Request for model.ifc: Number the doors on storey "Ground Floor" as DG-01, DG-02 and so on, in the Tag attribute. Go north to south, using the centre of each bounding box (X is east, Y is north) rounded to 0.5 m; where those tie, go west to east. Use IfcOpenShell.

First a look at what the model holds.

```python
import ifcopenshell
import ifcopenshell.util.element
import ifcopenshell.util.placement

model = ifcopenshell.open("model.ifc")
print(model.schema)
storey = next(s for s in model.by_type("IfcBuildingStorey") if s.Name == "Ground Floor")
doors = [e for e in ifcopenshell.util.element.get_decomposition(storey) if e.is_a("IfcDoor")]
for e in sorted(doors, key=lambda e: e.id()):
    origin = ifcopenshell.util.placement.get_local_placement(e.ObjectPlacement)[:3, 3]
    print(e.id(), e.Tag, e.Name, origin.round(2) + 0.0, sep=" | ")
```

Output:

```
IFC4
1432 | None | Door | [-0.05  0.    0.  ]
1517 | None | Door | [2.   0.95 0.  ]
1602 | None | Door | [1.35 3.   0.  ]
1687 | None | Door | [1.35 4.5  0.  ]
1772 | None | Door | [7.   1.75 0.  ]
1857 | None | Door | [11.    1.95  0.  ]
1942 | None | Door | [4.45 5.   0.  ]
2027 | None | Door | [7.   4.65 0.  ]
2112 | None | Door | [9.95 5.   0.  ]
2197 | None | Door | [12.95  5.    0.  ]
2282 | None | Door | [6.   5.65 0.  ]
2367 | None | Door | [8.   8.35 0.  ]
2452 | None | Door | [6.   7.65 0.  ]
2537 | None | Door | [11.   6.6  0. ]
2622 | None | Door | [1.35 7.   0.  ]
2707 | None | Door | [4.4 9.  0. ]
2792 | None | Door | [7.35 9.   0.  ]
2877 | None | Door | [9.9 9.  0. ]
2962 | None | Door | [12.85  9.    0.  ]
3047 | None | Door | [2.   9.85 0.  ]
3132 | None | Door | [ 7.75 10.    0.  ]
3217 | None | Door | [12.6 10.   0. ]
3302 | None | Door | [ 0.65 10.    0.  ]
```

```python
import ifcopenshell
import ifcopenshell.geom
import ifcopenshell.util.element
import ifcopenshell.util.shape

model = ifcopenshell.open("model.ifc")
settings = ifcopenshell.geom.settings()
settings.set("use-world-coords", True)


def centre(element):
    shape = ifcopenshell.geom.create_shape(settings, element)
    return ifcopenshell.util.shape.get_bbox_centroid(shape.geometry)


storey = next(s for s in model.by_type("IfcBuildingStorey") if s.Name == "Ground Floor")
doors = [e for e in ifcopenshell.util.element.get_decomposition(storey) if e.is_a("IfcDoor")]

# Insertion points can sit at a corner or the storey origin, so sort by the geometry (in metres).
centres = {e: centre(e) for e in doors}
doors.sort(key=lambda e: (-round(centres[e][1] / 0.5), centres[e][0]))

for i, e in enumerate(doors, start=1):
    number = f"DG-{i:02d}"
    e.Tag = number
    print(e.id(), number)

model.write("model_updated.ifc")
```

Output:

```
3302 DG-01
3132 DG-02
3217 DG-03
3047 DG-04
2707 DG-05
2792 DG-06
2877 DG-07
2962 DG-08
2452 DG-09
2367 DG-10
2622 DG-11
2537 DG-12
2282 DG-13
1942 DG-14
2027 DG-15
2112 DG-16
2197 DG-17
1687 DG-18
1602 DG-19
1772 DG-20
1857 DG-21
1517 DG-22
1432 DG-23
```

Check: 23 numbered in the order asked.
